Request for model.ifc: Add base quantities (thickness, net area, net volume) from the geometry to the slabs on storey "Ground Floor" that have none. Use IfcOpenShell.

First a look at what the model holds.

```python
import ifcopenshell
import ifcopenshell.util.element
import ifcopenshell.util.unit

model = ifcopenshell.open("model.ifc")
print(model.schema)
for unit_type in ("LENGTHUNIT", "AREAUNIT", "VOLUMEUNIT"):
    print(unit_type, ifcopenshell.util.unit.calculate_unit_scale(model, unit_type))
storey = next(s for s in model.by_type("IfcBuildingStorey") if s.Name == "Ground Floor")
slabs = [e for e in ifcopenshell.util.element.get_decomposition(storey) if e.is_a("IfcSlab")]
for e in sorted(slabs, key=lambda e: e.id()):
    print(e.id(), e.is_a(), e.Name, list(ifcopenshell.util.element.get_psets(e, qtos_only=True)), sep=" | ")
```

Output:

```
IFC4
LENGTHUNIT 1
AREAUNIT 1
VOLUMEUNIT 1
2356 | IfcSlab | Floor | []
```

```python
import ifcopenshell
import ifcopenshell.api.pset
import ifcopenshell.geom
import ifcopenshell.util.element
import ifcopenshell.util.shape
import ifcopenshell.util.unit

model = ifcopenshell.open("model.ifc")
unit_scale = ifcopenshell.util.unit.calculate_unit_scale(model)
area_scale = ifcopenshell.util.unit.calculate_unit_scale(model, "AREAUNIT")
volume_scale = ifcopenshell.util.unit.calculate_unit_scale(model, "VOLUMEUNIT")
settings = ifcopenshell.geom.settings()

storey = next(s for s in model.by_type("IfcBuildingStorey") if s.Name == "Ground Floor")
slabs = [e for e in ifcopenshell.util.element.get_decomposition(storey) if e.is_a("IfcSlab")]

for e in sorted(slabs, key=lambda e: e.id()):
    if ifcopenshell.util.element.get_psets(e, qtos_only=True, should_inherit=False):
        continue
    # Geometry comes back in metres, in the element's own axes.
    shape = ifcopenshell.geom.create_shape(settings, e)
    values = {
        "Width": ifcopenshell.util.shape.get_z(shape.geometry) / unit_scale,
        "NetArea": ifcopenshell.util.shape.get_footprint_area(shape.geometry) / area_scale,
        "NetVolume": ifcopenshell.util.shape.get_volume(shape.geometry) / volume_scale,
    }
    qto = ifcopenshell.api.pset.add_qto(model, product=e, name="Qto_SlabBaseQuantities")
    ifcopenshell.api.pset.edit_qto(model, qto=qto, properties=values)
    print(e.id(), {k: round(v, 3) for k, v in values.items()})

model.write("model_rev.ifc")
```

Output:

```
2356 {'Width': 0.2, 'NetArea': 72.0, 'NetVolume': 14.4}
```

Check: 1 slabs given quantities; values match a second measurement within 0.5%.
